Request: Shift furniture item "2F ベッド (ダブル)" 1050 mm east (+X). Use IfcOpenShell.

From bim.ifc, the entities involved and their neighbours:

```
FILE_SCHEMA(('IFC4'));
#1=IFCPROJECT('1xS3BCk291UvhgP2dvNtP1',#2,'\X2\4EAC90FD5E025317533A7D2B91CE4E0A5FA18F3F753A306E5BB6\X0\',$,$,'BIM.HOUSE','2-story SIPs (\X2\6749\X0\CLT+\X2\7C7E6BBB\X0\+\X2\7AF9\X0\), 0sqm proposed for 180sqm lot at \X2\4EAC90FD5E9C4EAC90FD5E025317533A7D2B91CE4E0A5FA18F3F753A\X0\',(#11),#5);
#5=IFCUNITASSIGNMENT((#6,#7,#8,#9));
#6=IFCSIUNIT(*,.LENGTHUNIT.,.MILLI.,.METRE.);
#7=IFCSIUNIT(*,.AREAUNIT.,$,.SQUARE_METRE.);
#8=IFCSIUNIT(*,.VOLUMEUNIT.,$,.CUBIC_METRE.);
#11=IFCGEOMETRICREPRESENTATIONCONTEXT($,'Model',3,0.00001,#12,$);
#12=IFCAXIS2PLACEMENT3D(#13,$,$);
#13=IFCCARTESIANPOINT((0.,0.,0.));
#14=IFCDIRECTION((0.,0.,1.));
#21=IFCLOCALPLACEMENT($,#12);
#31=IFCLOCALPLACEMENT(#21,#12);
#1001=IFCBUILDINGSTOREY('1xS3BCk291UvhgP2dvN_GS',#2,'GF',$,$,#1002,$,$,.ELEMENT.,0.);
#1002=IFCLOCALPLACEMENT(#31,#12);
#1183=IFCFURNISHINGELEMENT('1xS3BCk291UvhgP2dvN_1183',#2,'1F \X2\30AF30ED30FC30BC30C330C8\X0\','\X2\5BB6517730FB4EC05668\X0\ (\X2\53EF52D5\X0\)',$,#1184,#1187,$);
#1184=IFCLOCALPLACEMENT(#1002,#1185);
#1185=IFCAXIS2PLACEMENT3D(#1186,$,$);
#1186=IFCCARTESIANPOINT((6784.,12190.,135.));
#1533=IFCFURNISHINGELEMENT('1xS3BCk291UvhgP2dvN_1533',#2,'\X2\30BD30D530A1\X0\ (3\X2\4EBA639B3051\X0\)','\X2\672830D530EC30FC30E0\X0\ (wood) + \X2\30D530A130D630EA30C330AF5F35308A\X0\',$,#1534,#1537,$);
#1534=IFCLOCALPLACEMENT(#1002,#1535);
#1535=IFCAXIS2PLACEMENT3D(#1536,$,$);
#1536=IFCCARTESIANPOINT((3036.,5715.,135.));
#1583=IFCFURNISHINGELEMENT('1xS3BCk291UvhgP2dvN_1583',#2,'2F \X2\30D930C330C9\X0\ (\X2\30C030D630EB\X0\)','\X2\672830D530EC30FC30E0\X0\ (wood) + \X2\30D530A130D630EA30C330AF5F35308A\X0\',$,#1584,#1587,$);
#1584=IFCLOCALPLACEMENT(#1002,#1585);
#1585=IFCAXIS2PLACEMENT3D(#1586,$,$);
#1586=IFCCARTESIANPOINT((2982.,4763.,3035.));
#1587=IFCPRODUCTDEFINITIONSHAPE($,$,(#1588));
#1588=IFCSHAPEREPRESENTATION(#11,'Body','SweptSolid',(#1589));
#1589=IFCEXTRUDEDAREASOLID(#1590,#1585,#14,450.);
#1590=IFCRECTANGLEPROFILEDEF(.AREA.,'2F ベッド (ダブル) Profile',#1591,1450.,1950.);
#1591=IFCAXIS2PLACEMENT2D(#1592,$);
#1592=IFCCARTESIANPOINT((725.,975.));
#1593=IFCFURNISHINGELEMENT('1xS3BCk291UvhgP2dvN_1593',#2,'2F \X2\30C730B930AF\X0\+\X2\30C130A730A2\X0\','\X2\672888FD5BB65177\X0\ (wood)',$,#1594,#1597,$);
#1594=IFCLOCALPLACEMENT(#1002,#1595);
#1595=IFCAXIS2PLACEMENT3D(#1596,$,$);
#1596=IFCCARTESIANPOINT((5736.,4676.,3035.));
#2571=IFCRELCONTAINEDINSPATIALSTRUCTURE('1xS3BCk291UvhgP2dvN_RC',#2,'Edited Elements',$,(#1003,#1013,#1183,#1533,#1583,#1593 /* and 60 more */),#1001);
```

```python
import ifcopenshell
import ifcopenshell.api.geometry
import ifcopenshell.util.placement

model = ifcopenshell.open("bim.ifc")

item = model.by_id(1583)
matrix = ifcopenshell.util.placement.get_local_placement(item.ObjectPlacement)
matrix[0, 3] += 1050.0
ifcopenshell.api.geometry.edit_object_placement(model, product=item, matrix=matrix, is_si=False)

print(ifcopenshell.util.placement.get_local_placement(item.ObjectPlacement).round(3) + 0.0)

model.write("bim_updated.ifc")
```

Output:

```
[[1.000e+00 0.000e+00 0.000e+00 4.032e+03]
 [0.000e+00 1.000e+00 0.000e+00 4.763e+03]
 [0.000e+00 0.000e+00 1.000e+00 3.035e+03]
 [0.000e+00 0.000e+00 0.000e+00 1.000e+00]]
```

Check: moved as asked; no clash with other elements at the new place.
